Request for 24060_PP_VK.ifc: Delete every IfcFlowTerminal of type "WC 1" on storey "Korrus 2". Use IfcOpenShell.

First a look at what the model holds.

```python
import ifcopenshell
import ifcopenshell.util.element

model = ifcopenshell.open("24060_PP_VK.ifc")
print(model.schema)
storey = next(s for s in model.by_type("IfcBuildingStorey") if s.Name == "Korrus 2")
terminals = [e for e in ifcopenshell.util.element.get_decomposition(storey) if e.is_a("IfcFlowTerminal")]
seen = {}
for e in terminals:
    element_type = ifcopenshell.util.element.get_type(e)
    name = element_type.Name if element_type not in (None, e) else None
    seen[name] = seen.get(name, 0) + 1
for name, count in sorted(seen.items(), key=str):
    print(count, "x", name)
```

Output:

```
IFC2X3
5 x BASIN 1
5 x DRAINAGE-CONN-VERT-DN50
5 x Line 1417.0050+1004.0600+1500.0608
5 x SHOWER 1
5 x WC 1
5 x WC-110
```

```python
import ifcopenshell
import ifcopenshell.api.root
import ifcopenshell.util.element

model = ifcopenshell.open("24060_PP_VK.ifc")

storey = next(s for s in model.by_type("IfcBuildingStorey") if s.Name == "Korrus 2")
terminals = [e for e in ifcopenshell.util.element.get_decomposition(storey) if e.is_a("IfcFlowTerminal")]
targets = [e for e in terminals if (t := ifcopenshell.util.element.get_type(e)) not in (None, e) and t.Name == "WC 1"]

for e in targets:
    ifcopenshell.api.root.remove_product(model, product=e)
print(len(targets), "removed")

model.write("24060_PP_VK_edited.ifc")
```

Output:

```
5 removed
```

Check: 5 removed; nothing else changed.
